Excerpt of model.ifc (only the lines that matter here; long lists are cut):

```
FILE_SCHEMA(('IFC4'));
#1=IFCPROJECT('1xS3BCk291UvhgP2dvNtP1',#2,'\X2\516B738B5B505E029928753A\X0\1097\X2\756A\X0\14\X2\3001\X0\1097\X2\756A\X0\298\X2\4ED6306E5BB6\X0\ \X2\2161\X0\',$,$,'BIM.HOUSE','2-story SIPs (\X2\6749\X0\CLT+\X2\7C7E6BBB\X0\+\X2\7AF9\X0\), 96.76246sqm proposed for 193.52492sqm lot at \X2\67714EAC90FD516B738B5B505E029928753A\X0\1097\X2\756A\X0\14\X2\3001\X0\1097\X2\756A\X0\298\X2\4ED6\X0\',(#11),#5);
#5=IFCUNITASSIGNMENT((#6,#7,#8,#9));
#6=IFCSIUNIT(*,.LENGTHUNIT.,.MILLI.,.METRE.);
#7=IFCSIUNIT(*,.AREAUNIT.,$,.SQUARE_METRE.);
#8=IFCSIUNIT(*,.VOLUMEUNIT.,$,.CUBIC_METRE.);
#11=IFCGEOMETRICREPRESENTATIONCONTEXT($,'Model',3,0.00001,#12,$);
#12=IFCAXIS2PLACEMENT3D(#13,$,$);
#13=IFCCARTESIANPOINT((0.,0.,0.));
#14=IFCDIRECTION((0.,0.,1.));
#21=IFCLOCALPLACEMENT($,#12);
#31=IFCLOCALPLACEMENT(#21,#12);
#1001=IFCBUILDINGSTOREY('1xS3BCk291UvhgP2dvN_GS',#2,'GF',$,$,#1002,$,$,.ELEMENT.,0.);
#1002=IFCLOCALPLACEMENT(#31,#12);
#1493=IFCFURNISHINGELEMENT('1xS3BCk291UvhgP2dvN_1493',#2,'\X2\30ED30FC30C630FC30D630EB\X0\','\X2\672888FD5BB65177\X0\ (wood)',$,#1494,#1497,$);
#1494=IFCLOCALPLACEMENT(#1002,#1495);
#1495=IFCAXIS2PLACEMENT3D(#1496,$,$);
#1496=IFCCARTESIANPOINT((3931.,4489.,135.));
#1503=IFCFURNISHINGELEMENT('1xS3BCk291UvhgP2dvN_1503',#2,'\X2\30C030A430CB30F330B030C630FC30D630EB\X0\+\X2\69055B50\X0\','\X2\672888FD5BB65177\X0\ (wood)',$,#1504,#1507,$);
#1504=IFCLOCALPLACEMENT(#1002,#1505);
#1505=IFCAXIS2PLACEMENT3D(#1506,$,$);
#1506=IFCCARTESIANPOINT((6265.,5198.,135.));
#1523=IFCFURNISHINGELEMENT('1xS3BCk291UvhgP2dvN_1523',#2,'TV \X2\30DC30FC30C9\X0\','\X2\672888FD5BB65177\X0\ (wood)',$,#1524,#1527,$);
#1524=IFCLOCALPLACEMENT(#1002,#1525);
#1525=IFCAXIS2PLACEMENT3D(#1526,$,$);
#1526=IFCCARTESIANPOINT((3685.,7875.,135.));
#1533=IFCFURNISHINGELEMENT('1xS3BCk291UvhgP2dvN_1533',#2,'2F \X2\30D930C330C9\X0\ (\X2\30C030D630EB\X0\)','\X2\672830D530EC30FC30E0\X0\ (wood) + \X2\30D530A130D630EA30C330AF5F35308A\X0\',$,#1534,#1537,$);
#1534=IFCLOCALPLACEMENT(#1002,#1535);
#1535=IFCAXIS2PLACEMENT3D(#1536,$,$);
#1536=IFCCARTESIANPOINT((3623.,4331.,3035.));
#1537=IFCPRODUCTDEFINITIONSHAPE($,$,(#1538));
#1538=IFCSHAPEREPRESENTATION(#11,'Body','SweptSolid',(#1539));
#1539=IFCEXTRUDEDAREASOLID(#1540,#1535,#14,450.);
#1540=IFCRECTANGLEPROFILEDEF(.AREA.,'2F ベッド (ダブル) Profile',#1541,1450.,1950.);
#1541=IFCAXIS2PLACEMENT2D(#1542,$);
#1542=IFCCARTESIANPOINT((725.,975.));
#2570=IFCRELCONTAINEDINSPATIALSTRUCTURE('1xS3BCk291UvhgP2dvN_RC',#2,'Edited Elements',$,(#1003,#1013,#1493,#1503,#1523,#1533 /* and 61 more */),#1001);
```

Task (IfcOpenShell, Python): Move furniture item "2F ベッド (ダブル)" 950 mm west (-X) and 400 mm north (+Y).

```python
import ifcopenshell
import ifcopenshell.api.geometry
import ifcopenshell.util.placement
import ifcopenshell.util.unit

model = ifcopenshell.open("model.ifc")
unit_scale = ifcopenshell.util.unit.calculate_unit_scale(model)

item = model.by_guid("1xS3BCk291UvhgP2dvN_1533")
matrix = ifcopenshell.util.placement.get_local_placement(item.ObjectPlacement)
matrix[0, 3] -= 0.95 / unit_scale
matrix[1, 3] += 0.4 / unit_scale
ifcopenshell.api.geometry.edit_object_placement(model, product=item, matrix=matrix, is_si=False)

print(ifcopenshell.util.placement.get_local_placement(item.ObjectPlacement).round(3) + 0.0)

model.write("model_edited.ifc")
```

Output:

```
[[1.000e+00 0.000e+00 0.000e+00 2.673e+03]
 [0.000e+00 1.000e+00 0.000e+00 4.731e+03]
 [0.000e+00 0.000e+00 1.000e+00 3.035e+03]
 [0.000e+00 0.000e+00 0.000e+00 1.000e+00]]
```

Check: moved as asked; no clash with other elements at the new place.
